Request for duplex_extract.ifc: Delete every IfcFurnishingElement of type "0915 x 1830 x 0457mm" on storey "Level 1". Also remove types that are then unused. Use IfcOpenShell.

First a look at what the model holds.

```python
import ifcopenshell
import ifcopenshell.util.element

model = ifcopenshell.open("duplex_extract.ifc")
print(model.schema)
storey = next(s for s in model.by_type("IfcBuildingStorey") if s.Name == "Level 1")
furniture = [e for e in ifcopenshell.util.element.get_decomposition(storey) if e.is_a("IfcFurnishingElement")]
seen = {}
for e in furniture:
    element_type = ifcopenshell.util.element.get_type(e)
    name = element_type.Name if element_type not in (None, e) else None
    seen[name] = seen.get(name, 0) + 1
for name, count in sorted(seen.items(), key=str):
    print(count, "x", name)
```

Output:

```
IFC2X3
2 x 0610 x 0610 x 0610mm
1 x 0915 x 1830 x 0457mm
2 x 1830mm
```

```python
import ifcopenshell
import ifcopenshell.api.root
import ifcopenshell.util.element

model = ifcopenshell.open("duplex_extract.ifc")

storey = next(s for s in model.by_type("IfcBuildingStorey") if s.Name == "Level 1")
furniture = [e for e in ifcopenshell.util.element.get_decomposition(storey) if e.is_a("IfcFurnishingElement")]
targets = [e for e in furniture if (t := ifcopenshell.util.element.get_type(e)) not in (None, e) and t.Name == "0915 x 1830 x 0457mm"]
types = {ifcopenshell.util.element.get_type(e) for e in targets} - {None, *targets}

for e in targets:
    ifcopenshell.api.root.remove_product(model, product=e)
print(len(targets), "removed")

unused = [t for t in types if not ifcopenshell.util.element.get_types(t)]
for t in unused:
    ifcopenshell.api.root.remove_product(model, product=t)
print(len(unused), "unused types removed")

model.write("duplex_extract_edited.ifc")
```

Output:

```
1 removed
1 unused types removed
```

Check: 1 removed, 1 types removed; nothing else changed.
